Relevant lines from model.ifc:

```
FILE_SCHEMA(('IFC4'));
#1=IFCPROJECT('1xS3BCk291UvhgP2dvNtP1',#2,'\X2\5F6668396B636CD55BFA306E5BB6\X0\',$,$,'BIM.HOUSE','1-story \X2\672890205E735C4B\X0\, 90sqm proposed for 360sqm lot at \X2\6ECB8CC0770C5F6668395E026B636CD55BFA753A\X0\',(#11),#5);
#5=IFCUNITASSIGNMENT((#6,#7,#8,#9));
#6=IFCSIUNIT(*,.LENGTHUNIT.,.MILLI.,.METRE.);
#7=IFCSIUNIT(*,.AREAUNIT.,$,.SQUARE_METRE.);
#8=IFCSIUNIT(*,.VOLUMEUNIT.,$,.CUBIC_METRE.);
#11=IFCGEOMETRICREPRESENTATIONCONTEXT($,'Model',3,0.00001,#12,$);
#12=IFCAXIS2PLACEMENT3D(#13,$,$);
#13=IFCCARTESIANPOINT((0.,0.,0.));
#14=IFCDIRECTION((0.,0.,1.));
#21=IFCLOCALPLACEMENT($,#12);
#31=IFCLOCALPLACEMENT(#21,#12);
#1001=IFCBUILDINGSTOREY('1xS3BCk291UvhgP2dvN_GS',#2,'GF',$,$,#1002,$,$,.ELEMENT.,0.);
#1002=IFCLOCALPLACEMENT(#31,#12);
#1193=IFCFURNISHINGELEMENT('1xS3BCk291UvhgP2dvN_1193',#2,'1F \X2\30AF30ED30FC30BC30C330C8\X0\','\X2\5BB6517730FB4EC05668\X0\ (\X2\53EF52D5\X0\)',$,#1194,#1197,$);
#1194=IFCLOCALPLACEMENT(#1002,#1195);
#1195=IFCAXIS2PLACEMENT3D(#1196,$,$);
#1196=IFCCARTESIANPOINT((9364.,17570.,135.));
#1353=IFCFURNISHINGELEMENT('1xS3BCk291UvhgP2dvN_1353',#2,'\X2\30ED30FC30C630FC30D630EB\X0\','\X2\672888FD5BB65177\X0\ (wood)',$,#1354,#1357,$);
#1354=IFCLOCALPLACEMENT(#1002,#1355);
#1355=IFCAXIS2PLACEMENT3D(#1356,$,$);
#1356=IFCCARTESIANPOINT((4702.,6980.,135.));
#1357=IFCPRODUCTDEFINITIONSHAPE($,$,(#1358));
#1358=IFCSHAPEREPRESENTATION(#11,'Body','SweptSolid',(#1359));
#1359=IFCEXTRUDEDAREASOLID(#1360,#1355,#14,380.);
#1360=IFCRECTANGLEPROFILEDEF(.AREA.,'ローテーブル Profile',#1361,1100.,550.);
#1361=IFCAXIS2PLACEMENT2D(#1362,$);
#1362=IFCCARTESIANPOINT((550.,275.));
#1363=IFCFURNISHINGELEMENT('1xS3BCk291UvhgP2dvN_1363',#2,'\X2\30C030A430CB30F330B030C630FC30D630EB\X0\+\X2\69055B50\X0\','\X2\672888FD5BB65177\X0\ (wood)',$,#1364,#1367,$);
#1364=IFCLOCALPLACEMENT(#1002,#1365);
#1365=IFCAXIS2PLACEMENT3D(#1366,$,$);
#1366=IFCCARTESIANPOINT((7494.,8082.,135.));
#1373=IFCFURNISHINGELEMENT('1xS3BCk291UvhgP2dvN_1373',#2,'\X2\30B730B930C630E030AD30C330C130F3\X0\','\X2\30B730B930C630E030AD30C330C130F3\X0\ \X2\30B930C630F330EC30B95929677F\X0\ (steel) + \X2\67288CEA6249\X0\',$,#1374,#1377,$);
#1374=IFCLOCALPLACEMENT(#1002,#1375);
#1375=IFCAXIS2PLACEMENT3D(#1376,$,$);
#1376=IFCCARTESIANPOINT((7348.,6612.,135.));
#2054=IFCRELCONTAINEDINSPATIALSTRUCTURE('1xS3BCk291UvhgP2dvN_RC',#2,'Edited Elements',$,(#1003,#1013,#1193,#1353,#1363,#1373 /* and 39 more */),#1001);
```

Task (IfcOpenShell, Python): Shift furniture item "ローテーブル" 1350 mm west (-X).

```python
import ifcopenshell
import ifcopenshell.api.geometry
import ifcopenshell.util.placement
import ifcopenshell.util.unit

model = ifcopenshell.open("model.ifc")
unit_scale = ifcopenshell.util.unit.calculate_unit_scale(model)

item = model.by_guid("1xS3BCk291UvhgP2dvN_1353")
matrix = ifcopenshell.util.placement.get_local_placement(item.ObjectPlacement)
matrix[0, 3] -= 1.35 / unit_scale
ifcopenshell.api.geometry.edit_object_placement(model, product=item, matrix=matrix, is_si=False)

print(ifcopenshell.util.placement.get_local_placement(item.ObjectPlacement).round(3) + 0.0)

model.write("model_updated.ifc")
```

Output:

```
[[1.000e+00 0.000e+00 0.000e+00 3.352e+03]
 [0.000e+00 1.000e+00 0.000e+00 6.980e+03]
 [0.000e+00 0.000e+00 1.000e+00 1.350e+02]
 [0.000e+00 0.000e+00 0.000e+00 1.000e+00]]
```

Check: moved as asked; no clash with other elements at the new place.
